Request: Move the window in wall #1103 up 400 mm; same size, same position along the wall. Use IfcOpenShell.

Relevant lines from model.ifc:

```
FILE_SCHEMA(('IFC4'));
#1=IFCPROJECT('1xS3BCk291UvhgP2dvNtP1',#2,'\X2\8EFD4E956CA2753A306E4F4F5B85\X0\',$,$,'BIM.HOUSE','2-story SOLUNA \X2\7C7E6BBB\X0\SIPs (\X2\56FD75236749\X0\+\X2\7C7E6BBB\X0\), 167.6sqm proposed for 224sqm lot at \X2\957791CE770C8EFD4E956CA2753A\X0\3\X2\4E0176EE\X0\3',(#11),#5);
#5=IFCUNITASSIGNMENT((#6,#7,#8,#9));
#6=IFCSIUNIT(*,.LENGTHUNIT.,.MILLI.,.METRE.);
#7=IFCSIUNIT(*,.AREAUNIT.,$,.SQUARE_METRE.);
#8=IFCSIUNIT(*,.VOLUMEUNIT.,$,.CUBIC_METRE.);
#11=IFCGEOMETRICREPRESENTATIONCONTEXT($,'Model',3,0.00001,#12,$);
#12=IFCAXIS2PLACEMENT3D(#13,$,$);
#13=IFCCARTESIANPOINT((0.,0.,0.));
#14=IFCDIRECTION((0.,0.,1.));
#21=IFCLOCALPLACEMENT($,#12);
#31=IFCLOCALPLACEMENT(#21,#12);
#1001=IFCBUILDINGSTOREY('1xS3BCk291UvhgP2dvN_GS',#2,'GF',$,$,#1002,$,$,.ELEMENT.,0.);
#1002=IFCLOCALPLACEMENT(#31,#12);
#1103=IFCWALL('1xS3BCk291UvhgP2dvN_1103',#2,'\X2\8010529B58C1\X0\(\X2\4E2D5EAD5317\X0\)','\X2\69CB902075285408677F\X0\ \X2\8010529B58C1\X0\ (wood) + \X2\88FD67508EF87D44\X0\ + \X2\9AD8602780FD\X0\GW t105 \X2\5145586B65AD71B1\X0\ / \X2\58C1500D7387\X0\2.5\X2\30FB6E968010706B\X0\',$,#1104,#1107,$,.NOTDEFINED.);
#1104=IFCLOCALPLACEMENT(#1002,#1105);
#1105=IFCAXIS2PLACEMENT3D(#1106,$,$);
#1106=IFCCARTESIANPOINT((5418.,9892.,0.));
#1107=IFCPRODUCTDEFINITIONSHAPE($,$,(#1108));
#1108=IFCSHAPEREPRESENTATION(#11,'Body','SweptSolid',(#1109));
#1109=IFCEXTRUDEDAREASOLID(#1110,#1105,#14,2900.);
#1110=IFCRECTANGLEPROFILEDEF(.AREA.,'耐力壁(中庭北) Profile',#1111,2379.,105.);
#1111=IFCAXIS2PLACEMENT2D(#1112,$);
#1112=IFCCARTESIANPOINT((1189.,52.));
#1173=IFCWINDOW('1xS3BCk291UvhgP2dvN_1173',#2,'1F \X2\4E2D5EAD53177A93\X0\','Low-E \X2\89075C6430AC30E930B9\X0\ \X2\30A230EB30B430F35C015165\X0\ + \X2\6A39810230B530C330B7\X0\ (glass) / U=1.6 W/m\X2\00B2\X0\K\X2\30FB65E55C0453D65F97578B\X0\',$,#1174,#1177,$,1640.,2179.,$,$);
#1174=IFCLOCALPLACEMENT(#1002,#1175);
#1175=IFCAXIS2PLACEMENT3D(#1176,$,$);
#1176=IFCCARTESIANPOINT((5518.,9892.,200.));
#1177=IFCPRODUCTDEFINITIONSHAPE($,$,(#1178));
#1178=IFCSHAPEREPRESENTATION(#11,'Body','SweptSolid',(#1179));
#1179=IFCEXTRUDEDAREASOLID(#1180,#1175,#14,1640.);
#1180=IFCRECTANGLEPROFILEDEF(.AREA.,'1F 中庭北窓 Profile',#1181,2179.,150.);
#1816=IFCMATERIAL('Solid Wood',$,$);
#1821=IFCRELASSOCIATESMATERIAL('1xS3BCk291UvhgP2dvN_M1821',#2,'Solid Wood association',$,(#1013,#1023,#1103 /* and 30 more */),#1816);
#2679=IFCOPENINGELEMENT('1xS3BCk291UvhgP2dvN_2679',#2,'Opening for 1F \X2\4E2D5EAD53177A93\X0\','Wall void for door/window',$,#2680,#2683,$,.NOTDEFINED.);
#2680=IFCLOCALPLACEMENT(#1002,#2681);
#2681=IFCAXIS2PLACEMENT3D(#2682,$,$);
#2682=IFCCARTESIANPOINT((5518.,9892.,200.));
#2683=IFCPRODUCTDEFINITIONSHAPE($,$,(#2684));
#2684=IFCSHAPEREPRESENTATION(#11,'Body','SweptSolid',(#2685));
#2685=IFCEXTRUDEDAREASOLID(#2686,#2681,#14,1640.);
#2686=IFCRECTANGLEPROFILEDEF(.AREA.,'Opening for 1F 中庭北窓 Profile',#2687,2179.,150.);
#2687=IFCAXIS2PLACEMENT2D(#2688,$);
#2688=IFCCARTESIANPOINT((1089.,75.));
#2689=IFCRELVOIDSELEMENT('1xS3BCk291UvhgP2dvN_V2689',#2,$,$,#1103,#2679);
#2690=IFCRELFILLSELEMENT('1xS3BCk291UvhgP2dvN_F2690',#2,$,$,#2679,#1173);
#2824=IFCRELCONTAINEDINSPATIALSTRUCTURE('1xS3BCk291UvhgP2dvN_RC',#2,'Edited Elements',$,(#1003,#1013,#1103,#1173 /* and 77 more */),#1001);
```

```python
import numpy as np
import ifcopenshell
import ifcopenshell.api.geometry
import ifcopenshell.util.placement
import ifcopenshell.util.unit

model = ifcopenshell.open("model.ifc")
unit_scale = ifcopenshell.util.unit.calculate_unit_scale(model)

window = model.by_guid("1xS3BCk291UvhgP2dvN_1173")
opening = window.FillsVoids[0].RelatingOpeningElement
dz = 400.0

shift = np.array([0.0, 0.0, dz])
# The window is not placed relative to its opening, so move both.
for product in (opening, window):
    matrix = ifcopenshell.util.placement.get_local_placement(product.ObjectPlacement)
    matrix[:3, 3] += shift
    ifcopenshell.api.geometry.edit_object_placement(model, product=product, matrix=matrix, is_si=False)

print(f"moved by {dz * unit_scale:+.3f} m")

model.write("model-out.ifc")
```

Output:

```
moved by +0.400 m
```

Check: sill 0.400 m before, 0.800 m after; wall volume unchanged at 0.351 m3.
